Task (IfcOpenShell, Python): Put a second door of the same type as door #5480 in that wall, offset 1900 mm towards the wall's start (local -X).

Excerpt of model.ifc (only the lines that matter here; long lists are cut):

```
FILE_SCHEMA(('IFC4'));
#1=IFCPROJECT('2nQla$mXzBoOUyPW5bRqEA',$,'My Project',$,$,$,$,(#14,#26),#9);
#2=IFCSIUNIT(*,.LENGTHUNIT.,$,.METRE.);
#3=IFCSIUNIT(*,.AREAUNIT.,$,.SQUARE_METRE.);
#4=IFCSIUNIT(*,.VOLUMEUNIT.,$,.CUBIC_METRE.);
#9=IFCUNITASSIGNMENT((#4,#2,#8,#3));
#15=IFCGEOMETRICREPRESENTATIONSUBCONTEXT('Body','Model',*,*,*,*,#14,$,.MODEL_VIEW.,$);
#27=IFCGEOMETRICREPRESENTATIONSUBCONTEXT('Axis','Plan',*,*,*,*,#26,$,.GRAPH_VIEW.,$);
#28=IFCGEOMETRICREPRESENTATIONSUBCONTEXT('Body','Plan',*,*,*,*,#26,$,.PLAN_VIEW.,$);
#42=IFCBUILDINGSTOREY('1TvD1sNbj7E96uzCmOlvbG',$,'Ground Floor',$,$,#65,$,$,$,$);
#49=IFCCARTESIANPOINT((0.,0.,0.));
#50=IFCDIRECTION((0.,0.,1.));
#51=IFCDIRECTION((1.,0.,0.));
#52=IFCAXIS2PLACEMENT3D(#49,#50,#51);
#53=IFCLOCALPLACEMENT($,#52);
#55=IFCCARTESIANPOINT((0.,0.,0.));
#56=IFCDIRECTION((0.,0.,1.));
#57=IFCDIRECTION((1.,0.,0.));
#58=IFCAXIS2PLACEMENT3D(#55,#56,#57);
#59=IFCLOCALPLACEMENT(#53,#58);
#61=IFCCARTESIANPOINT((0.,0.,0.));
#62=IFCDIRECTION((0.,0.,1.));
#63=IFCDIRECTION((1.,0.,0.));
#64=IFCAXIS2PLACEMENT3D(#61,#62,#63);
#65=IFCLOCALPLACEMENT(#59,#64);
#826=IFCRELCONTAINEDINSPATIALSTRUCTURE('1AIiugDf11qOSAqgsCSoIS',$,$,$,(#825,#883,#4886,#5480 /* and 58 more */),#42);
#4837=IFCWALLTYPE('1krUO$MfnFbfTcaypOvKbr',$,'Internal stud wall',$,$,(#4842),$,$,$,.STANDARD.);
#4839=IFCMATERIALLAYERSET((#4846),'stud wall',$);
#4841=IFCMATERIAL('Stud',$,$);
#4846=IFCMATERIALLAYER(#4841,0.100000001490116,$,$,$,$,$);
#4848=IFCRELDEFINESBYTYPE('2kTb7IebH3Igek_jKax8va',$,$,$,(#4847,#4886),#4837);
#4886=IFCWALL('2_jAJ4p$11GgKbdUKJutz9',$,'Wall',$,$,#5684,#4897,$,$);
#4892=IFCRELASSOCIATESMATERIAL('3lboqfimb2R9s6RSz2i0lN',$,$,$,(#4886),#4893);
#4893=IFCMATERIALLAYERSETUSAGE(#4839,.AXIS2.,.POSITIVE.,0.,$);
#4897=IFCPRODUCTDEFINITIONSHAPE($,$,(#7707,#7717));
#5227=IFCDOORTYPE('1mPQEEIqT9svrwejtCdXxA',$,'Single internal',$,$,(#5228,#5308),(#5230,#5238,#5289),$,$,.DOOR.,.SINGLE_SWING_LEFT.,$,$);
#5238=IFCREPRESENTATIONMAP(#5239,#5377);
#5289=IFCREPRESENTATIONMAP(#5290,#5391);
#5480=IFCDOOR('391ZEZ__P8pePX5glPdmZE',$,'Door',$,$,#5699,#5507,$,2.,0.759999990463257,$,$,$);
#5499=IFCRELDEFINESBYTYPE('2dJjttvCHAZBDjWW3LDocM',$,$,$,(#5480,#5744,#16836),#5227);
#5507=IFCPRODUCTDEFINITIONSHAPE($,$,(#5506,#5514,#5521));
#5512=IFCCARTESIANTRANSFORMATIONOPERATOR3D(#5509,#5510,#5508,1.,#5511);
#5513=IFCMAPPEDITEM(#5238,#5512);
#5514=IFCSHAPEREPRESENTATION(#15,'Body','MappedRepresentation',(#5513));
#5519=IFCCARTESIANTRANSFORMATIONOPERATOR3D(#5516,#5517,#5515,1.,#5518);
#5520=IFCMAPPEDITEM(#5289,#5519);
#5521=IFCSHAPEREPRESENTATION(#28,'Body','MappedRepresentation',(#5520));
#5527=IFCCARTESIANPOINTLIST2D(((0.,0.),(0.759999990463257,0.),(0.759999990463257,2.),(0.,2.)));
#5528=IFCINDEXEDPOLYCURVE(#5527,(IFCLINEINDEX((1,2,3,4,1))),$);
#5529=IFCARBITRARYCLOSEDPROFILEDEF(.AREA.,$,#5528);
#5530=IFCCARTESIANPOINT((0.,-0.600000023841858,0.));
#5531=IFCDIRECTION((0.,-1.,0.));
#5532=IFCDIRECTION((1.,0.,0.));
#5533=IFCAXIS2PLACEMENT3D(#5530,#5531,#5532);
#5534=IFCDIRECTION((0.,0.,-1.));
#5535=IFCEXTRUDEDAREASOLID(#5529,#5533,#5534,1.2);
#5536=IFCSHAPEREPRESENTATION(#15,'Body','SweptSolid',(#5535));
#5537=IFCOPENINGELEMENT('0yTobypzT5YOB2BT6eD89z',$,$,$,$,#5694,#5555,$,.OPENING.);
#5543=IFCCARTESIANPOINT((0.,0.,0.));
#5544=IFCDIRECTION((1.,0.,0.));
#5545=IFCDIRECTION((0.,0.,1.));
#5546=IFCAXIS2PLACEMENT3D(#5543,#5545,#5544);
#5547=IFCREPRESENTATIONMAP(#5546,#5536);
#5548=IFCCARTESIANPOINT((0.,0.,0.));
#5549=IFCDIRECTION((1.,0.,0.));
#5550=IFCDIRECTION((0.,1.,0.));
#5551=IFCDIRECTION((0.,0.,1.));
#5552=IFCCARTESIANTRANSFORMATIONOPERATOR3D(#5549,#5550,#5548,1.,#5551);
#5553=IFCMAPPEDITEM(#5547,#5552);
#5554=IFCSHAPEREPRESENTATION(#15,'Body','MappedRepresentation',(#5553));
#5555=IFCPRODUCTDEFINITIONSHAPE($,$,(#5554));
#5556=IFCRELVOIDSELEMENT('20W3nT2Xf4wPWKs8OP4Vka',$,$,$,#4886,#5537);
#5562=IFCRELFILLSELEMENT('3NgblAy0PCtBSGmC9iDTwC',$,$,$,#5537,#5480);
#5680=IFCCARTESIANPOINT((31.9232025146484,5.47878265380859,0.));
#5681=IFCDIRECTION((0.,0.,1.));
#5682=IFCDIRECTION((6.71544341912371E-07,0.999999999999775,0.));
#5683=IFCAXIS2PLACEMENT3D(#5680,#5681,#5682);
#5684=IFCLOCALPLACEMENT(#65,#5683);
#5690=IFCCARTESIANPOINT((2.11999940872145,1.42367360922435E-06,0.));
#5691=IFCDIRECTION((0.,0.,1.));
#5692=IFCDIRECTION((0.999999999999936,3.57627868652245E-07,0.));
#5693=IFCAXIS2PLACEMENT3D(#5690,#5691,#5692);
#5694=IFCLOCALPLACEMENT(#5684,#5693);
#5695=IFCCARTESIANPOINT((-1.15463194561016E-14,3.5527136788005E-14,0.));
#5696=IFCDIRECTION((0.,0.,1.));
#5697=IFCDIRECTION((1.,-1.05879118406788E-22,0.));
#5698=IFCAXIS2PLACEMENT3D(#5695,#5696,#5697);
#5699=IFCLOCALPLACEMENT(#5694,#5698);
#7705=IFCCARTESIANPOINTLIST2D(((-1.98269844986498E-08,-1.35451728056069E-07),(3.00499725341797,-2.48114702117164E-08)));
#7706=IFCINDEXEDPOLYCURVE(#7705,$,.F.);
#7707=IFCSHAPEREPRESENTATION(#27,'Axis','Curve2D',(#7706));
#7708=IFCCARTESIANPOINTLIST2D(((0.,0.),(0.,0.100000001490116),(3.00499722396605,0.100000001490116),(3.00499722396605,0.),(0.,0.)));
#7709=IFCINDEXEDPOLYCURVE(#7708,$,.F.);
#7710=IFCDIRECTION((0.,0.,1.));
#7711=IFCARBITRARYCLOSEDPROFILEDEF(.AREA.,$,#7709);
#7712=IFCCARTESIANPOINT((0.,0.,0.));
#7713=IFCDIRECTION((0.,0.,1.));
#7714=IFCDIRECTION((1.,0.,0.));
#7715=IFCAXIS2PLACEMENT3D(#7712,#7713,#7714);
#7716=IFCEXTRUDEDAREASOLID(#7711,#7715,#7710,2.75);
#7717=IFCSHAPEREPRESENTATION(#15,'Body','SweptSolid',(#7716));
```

```python
import ifcopenshell
import ifcopenshell.api.feature
import ifcopenshell.api.geometry
import ifcopenshell.api.root
import ifcopenshell.geom
import ifcopenshell.util.element
import ifcopenshell.util.placement
import ifcopenshell.util.shape

model = ifcopenshell.open("model.ifc")
settings = ifcopenshell.geom.settings()


def volume(element):
    """Net volume in cubic metres, openings subtracted."""
    shape = ifcopenshell.geom.create_shape(settings, element)
    return ifcopenshell.util.shape.get_volume(shape.geometry)


door = model.by_guid("391ZEZ__P8pePX5glPdmZE")
opening = door.FillsVoids[0].RelatingOpeningElement
wall = opening.VoidsElements[0].RelatingBuildingElement
before = volume(wall)
shift = ifcopenshell.util.placement.get_local_placement(wall.ObjectPlacement)[:3, 0] * -1.9

# copy_class copies the void relationship, type, container and properties, but no geometry.
new_opening = ifcopenshell.api.root.copy_class(model, product=opening)
new_opening.Representation = ifcopenshell.util.element.copy_deep(
    model, opening.Representation, exclude=["IfcGeometricRepresentationContext", "IfcRepresentationMap"]
)
new_door = ifcopenshell.api.root.copy_class(model, product=door)
new_door.Representation = ifcopenshell.util.element.copy_deep(
    model, door.Representation, exclude=["IfcGeometricRepresentationContext", "IfcRepresentationMap"]
)
ifcopenshell.api.feature.add_filling(model, opening=new_opening, element=new_door)

for old, new in ((opening, new_opening), (door, new_door)):
    matrix = ifcopenshell.util.placement.get_local_placement(old.ObjectPlacement)
    matrix[:3, 3] += shift
    ifcopenshell.api.geometry.edit_object_placement(model, product=new, matrix=matrix, is_si=False)

after = volume(wall)

print(f"wall volume {before:.3f} -> {after:.3f} m3")

model.write("model_edited.ifc")
```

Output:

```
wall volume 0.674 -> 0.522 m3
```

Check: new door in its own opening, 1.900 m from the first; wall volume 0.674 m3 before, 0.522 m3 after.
